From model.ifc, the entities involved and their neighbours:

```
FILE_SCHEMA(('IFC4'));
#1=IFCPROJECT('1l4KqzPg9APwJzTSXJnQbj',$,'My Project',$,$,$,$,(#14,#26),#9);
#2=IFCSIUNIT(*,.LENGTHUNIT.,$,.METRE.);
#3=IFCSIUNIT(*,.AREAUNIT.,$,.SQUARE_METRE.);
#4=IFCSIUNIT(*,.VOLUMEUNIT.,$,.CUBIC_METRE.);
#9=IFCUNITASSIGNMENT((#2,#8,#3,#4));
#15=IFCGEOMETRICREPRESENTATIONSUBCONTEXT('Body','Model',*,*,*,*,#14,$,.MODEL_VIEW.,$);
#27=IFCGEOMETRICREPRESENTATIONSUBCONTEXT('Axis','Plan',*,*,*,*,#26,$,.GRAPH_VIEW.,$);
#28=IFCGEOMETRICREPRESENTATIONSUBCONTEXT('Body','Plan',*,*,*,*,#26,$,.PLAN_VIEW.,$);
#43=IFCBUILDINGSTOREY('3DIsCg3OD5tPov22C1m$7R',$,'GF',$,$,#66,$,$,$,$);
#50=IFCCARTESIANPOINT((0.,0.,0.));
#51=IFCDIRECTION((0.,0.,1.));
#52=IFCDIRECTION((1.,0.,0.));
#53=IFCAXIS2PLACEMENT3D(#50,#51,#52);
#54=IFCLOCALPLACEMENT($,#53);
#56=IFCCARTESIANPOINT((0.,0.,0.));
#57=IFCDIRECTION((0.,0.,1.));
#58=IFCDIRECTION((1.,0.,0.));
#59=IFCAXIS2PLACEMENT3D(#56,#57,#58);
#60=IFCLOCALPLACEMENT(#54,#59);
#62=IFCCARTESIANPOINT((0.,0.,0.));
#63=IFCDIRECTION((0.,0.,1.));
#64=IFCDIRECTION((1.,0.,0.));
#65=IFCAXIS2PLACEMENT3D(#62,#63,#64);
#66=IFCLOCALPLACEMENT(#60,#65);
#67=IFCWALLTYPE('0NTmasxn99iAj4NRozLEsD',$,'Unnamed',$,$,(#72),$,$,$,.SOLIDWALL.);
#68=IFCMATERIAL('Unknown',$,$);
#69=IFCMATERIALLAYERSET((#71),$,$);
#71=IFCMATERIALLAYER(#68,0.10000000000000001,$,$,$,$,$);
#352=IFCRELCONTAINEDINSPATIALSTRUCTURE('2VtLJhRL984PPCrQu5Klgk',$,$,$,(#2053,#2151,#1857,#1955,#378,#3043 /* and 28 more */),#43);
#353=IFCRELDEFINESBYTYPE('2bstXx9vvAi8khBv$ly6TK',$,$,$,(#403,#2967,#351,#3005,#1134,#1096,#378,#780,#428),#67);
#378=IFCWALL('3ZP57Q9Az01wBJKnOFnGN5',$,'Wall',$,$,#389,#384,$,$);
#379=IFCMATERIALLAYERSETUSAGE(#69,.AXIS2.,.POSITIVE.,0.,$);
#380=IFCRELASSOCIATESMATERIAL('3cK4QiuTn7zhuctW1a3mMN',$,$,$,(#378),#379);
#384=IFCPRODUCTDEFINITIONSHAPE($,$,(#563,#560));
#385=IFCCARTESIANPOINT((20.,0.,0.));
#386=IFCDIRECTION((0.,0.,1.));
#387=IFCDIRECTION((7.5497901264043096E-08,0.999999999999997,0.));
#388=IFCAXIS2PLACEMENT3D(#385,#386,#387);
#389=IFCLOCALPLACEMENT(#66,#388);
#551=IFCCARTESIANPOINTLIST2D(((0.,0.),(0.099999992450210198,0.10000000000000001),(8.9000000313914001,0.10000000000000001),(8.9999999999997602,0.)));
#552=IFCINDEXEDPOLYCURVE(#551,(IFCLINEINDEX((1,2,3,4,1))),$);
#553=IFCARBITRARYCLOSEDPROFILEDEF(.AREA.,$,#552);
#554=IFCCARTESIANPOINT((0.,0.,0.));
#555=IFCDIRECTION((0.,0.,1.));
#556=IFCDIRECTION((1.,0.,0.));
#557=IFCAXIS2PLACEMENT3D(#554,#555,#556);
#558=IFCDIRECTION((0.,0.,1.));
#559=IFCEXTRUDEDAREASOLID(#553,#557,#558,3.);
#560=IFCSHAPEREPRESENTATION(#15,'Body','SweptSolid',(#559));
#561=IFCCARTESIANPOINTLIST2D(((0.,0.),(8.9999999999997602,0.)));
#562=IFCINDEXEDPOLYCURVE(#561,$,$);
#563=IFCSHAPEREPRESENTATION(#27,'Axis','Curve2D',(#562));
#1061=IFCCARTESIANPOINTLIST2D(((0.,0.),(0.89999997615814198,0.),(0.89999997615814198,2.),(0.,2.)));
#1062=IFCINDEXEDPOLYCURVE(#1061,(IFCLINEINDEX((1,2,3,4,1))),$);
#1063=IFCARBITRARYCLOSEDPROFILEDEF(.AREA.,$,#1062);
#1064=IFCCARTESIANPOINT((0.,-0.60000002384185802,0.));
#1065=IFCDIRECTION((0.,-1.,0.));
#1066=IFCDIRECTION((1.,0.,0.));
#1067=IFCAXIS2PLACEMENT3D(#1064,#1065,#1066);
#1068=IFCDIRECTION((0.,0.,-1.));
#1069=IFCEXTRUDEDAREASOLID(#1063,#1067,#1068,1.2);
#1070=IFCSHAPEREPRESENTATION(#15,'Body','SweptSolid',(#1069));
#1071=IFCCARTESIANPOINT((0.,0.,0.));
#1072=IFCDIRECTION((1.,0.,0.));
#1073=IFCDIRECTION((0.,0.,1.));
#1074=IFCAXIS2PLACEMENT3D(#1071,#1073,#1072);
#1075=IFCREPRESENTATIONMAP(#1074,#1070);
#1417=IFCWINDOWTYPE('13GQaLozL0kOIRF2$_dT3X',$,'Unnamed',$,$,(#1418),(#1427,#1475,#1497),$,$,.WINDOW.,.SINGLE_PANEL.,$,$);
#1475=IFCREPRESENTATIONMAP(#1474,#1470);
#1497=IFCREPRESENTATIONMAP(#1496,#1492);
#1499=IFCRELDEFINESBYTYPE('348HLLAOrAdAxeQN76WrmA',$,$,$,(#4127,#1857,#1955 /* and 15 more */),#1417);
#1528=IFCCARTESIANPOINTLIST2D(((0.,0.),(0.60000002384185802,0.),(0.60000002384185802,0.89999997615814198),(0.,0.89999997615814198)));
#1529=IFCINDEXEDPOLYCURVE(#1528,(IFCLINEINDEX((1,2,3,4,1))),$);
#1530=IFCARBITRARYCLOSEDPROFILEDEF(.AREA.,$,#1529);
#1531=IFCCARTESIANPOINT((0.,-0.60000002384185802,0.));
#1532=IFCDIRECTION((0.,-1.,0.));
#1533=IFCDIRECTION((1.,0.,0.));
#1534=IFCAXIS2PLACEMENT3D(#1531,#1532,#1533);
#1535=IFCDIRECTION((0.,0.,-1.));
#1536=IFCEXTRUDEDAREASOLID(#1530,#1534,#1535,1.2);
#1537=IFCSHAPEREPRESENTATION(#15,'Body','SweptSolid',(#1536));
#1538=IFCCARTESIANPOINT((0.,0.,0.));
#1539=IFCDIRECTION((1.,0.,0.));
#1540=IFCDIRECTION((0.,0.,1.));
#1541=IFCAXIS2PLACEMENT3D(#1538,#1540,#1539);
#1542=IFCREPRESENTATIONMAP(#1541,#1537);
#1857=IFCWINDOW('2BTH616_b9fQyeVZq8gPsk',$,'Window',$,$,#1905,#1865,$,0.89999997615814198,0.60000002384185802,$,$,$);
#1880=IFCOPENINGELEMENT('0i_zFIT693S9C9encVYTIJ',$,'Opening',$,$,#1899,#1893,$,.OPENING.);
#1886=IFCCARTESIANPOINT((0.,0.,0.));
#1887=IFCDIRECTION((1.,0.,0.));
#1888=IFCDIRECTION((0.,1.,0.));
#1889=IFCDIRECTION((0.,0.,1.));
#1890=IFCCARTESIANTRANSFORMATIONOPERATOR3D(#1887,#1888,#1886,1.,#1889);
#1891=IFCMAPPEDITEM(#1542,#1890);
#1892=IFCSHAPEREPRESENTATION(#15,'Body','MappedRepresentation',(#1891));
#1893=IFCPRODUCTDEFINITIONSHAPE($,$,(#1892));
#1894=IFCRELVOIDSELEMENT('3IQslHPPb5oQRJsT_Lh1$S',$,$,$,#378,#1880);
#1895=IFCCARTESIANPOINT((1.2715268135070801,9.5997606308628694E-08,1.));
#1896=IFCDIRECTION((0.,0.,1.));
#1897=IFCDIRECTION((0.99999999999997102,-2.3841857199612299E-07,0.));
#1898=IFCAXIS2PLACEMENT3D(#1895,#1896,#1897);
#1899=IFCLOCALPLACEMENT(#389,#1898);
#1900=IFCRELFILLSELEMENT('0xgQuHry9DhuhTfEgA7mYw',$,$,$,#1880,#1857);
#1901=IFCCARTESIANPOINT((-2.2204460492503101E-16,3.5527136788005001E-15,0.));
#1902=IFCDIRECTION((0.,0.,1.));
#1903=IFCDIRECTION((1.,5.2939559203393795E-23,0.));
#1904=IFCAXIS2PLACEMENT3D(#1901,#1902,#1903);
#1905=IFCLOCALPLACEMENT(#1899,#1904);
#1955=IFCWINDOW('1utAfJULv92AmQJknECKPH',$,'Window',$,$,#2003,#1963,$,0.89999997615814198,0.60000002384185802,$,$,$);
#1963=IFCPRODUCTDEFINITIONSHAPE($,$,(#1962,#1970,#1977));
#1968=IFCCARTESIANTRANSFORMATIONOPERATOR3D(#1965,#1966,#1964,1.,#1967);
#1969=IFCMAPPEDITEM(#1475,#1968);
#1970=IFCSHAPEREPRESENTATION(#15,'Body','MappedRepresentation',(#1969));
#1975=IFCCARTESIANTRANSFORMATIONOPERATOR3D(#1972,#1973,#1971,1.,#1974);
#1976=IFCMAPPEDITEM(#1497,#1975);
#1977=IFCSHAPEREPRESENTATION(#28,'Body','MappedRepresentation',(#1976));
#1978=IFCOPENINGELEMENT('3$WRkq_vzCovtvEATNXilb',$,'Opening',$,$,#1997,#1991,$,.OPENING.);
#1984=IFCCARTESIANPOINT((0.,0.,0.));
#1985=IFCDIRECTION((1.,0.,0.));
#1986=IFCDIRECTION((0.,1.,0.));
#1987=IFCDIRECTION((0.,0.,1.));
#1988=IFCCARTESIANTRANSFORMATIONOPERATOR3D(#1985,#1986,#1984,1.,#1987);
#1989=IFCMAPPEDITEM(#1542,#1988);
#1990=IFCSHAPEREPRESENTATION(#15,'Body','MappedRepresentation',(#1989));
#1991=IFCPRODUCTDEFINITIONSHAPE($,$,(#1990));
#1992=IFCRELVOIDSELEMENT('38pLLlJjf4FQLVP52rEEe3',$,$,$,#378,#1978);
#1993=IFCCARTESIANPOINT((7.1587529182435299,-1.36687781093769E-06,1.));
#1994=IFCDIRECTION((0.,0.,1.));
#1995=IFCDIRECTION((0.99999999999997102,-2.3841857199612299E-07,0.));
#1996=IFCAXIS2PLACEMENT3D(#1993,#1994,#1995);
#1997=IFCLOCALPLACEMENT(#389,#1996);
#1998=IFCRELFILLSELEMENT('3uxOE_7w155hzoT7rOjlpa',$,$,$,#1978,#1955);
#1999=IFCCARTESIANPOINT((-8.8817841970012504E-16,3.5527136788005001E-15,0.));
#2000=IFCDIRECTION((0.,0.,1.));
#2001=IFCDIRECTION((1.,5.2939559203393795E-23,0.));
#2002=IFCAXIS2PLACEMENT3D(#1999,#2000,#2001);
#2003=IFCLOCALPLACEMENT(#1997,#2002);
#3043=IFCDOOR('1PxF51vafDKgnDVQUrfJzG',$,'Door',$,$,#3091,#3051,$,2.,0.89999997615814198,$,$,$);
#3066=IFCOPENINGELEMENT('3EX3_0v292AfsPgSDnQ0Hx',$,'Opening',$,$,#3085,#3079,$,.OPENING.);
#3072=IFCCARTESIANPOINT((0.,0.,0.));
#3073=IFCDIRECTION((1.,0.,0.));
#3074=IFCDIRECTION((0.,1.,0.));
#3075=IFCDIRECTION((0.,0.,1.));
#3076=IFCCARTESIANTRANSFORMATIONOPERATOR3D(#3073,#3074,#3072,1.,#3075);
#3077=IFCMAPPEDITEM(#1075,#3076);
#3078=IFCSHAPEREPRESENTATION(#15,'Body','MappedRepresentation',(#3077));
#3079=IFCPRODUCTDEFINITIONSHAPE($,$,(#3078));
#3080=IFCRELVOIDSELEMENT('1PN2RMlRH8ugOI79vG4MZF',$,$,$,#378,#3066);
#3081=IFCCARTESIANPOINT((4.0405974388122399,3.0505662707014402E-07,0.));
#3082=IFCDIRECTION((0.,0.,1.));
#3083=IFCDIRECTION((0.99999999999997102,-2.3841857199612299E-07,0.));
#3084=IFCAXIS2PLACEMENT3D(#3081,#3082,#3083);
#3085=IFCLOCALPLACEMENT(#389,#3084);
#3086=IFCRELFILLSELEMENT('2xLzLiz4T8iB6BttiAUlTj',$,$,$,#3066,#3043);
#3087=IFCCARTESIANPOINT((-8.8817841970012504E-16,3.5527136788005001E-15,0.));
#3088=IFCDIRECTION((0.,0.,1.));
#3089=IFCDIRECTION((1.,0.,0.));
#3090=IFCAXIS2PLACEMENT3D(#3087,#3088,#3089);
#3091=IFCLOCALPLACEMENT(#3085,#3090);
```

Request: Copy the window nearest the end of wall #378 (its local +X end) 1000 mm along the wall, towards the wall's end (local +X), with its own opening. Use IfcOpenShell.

```python
import ifcopenshell
import ifcopenshell.api.feature
import ifcopenshell.api.geometry
import ifcopenshell.api.root
import ifcopenshell.geom
import ifcopenshell.util.element
import ifcopenshell.util.placement
import ifcopenshell.util.shape

model = ifcopenshell.open("model.ifc")
settings = ifcopenshell.geom.settings()


def volume(element):
    """Net volume in cubic metres, openings subtracted."""
    shape = ifcopenshell.geom.create_shape(settings, element)
    return ifcopenshell.util.shape.get_volume(shape.geometry)


window = model.by_guid("1utAfJULv92AmQJknECKPH")
opening = window.FillsVoids[0].RelatingOpeningElement
wall = opening.VoidsElements[0].RelatingBuildingElement
before = volume(wall)
shift = ifcopenshell.util.placement.get_local_placement(wall.ObjectPlacement)[:3, 0] * 1.0

# copy_class copies the void relationship, type, container and properties, but no geometry.
new_opening = ifcopenshell.api.root.copy_class(model, product=opening)
new_opening.Representation = ifcopenshell.util.element.copy_deep(
    model, opening.Representation, exclude=["IfcGeometricRepresentationContext", "IfcRepresentationMap"]
)
new_window = ifcopenshell.api.root.copy_class(model, product=window)
new_window.Representation = ifcopenshell.util.element.copy_deep(
    model, window.Representation, exclude=["IfcGeometricRepresentationContext", "IfcRepresentationMap"]
)
ifcopenshell.api.feature.add_filling(model, opening=new_opening, element=new_window)

for old, new in ((opening, new_opening), (window, new_window)):
    matrix = ifcopenshell.util.placement.get_local_placement(old.ObjectPlacement)
    matrix[:3, 3] += shift
    ifcopenshell.api.geometry.edit_object_placement(model, product=new, matrix=matrix, is_si=False)

after = volume(wall)

print(f"wall volume {before:.3f} -> {after:.3f} m3")

model.write("model_rev.ifc")
```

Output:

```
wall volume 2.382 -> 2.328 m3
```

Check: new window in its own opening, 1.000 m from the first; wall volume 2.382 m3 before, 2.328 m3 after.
